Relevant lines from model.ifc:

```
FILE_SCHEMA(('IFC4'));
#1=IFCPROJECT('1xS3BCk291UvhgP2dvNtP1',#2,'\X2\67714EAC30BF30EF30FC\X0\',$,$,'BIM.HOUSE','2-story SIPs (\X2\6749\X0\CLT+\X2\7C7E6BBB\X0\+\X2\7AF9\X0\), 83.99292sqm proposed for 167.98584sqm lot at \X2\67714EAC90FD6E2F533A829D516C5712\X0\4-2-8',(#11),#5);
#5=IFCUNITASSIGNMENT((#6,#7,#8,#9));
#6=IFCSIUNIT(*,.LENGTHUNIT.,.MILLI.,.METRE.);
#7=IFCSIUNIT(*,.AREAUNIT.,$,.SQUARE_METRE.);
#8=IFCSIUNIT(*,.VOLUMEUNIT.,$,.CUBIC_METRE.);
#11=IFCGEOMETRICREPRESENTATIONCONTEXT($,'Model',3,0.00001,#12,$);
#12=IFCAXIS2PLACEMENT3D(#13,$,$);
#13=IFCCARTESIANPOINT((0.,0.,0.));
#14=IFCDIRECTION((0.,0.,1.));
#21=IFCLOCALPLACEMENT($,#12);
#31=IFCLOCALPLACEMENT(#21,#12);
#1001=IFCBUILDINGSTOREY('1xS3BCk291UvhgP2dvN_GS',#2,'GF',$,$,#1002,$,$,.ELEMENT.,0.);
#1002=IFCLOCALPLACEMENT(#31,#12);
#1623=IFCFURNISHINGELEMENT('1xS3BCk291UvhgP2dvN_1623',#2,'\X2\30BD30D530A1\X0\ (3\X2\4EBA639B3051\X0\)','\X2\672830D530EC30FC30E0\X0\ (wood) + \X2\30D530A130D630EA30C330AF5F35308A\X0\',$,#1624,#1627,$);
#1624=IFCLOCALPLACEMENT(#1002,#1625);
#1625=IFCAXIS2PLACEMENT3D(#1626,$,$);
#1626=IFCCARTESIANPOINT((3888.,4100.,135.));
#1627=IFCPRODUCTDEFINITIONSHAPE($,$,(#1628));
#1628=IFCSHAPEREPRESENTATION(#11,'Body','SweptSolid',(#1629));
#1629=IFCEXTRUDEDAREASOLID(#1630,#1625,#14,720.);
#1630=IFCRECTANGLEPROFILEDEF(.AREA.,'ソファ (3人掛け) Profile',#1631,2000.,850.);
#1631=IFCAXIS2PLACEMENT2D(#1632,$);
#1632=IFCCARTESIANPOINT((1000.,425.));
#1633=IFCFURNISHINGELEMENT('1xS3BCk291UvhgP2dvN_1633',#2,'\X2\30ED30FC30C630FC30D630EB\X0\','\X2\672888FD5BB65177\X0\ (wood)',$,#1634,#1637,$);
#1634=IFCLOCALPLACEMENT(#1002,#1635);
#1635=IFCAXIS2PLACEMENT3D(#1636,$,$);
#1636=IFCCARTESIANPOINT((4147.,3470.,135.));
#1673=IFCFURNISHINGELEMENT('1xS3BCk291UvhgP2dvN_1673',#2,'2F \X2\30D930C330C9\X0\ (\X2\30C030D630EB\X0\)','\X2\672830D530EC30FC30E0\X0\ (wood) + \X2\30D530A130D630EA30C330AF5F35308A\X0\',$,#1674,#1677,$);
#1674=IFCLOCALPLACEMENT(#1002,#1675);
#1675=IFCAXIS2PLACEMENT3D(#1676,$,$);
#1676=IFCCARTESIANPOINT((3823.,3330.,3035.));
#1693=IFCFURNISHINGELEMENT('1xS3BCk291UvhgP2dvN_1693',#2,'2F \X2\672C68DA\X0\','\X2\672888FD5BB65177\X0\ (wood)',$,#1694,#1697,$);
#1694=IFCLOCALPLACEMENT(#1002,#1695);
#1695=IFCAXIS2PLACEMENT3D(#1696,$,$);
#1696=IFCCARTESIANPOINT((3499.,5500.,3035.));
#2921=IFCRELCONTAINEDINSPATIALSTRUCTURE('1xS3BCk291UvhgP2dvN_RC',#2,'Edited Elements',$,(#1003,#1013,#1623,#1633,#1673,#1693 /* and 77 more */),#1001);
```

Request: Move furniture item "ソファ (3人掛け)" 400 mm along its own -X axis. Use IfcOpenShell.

```python
import ifcopenshell
import ifcopenshell.api.geometry
import ifcopenshell.util.placement
import ifcopenshell.util.unit

model = ifcopenshell.open("model.ifc")
unit_scale = ifcopenshell.util.unit.calculate_unit_scale(model)

item = model.by_guid("1xS3BCk291UvhgP2dvN_1623")
matrix = ifcopenshell.util.placement.get_local_placement(item.ObjectPlacement)
matrix[:3, 3] -= matrix[:3, 0] * 0.4 / unit_scale
ifcopenshell.api.geometry.edit_object_placement(model, product=item, matrix=matrix, is_si=False)

print(ifcopenshell.util.placement.get_local_placement(item.ObjectPlacement).round(3) + 0.0)

model.write("model_rev.ifc")
```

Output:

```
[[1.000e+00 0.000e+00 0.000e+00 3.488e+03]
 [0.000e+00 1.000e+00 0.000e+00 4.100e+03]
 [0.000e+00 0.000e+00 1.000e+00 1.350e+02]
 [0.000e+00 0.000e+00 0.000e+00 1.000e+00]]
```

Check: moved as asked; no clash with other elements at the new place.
